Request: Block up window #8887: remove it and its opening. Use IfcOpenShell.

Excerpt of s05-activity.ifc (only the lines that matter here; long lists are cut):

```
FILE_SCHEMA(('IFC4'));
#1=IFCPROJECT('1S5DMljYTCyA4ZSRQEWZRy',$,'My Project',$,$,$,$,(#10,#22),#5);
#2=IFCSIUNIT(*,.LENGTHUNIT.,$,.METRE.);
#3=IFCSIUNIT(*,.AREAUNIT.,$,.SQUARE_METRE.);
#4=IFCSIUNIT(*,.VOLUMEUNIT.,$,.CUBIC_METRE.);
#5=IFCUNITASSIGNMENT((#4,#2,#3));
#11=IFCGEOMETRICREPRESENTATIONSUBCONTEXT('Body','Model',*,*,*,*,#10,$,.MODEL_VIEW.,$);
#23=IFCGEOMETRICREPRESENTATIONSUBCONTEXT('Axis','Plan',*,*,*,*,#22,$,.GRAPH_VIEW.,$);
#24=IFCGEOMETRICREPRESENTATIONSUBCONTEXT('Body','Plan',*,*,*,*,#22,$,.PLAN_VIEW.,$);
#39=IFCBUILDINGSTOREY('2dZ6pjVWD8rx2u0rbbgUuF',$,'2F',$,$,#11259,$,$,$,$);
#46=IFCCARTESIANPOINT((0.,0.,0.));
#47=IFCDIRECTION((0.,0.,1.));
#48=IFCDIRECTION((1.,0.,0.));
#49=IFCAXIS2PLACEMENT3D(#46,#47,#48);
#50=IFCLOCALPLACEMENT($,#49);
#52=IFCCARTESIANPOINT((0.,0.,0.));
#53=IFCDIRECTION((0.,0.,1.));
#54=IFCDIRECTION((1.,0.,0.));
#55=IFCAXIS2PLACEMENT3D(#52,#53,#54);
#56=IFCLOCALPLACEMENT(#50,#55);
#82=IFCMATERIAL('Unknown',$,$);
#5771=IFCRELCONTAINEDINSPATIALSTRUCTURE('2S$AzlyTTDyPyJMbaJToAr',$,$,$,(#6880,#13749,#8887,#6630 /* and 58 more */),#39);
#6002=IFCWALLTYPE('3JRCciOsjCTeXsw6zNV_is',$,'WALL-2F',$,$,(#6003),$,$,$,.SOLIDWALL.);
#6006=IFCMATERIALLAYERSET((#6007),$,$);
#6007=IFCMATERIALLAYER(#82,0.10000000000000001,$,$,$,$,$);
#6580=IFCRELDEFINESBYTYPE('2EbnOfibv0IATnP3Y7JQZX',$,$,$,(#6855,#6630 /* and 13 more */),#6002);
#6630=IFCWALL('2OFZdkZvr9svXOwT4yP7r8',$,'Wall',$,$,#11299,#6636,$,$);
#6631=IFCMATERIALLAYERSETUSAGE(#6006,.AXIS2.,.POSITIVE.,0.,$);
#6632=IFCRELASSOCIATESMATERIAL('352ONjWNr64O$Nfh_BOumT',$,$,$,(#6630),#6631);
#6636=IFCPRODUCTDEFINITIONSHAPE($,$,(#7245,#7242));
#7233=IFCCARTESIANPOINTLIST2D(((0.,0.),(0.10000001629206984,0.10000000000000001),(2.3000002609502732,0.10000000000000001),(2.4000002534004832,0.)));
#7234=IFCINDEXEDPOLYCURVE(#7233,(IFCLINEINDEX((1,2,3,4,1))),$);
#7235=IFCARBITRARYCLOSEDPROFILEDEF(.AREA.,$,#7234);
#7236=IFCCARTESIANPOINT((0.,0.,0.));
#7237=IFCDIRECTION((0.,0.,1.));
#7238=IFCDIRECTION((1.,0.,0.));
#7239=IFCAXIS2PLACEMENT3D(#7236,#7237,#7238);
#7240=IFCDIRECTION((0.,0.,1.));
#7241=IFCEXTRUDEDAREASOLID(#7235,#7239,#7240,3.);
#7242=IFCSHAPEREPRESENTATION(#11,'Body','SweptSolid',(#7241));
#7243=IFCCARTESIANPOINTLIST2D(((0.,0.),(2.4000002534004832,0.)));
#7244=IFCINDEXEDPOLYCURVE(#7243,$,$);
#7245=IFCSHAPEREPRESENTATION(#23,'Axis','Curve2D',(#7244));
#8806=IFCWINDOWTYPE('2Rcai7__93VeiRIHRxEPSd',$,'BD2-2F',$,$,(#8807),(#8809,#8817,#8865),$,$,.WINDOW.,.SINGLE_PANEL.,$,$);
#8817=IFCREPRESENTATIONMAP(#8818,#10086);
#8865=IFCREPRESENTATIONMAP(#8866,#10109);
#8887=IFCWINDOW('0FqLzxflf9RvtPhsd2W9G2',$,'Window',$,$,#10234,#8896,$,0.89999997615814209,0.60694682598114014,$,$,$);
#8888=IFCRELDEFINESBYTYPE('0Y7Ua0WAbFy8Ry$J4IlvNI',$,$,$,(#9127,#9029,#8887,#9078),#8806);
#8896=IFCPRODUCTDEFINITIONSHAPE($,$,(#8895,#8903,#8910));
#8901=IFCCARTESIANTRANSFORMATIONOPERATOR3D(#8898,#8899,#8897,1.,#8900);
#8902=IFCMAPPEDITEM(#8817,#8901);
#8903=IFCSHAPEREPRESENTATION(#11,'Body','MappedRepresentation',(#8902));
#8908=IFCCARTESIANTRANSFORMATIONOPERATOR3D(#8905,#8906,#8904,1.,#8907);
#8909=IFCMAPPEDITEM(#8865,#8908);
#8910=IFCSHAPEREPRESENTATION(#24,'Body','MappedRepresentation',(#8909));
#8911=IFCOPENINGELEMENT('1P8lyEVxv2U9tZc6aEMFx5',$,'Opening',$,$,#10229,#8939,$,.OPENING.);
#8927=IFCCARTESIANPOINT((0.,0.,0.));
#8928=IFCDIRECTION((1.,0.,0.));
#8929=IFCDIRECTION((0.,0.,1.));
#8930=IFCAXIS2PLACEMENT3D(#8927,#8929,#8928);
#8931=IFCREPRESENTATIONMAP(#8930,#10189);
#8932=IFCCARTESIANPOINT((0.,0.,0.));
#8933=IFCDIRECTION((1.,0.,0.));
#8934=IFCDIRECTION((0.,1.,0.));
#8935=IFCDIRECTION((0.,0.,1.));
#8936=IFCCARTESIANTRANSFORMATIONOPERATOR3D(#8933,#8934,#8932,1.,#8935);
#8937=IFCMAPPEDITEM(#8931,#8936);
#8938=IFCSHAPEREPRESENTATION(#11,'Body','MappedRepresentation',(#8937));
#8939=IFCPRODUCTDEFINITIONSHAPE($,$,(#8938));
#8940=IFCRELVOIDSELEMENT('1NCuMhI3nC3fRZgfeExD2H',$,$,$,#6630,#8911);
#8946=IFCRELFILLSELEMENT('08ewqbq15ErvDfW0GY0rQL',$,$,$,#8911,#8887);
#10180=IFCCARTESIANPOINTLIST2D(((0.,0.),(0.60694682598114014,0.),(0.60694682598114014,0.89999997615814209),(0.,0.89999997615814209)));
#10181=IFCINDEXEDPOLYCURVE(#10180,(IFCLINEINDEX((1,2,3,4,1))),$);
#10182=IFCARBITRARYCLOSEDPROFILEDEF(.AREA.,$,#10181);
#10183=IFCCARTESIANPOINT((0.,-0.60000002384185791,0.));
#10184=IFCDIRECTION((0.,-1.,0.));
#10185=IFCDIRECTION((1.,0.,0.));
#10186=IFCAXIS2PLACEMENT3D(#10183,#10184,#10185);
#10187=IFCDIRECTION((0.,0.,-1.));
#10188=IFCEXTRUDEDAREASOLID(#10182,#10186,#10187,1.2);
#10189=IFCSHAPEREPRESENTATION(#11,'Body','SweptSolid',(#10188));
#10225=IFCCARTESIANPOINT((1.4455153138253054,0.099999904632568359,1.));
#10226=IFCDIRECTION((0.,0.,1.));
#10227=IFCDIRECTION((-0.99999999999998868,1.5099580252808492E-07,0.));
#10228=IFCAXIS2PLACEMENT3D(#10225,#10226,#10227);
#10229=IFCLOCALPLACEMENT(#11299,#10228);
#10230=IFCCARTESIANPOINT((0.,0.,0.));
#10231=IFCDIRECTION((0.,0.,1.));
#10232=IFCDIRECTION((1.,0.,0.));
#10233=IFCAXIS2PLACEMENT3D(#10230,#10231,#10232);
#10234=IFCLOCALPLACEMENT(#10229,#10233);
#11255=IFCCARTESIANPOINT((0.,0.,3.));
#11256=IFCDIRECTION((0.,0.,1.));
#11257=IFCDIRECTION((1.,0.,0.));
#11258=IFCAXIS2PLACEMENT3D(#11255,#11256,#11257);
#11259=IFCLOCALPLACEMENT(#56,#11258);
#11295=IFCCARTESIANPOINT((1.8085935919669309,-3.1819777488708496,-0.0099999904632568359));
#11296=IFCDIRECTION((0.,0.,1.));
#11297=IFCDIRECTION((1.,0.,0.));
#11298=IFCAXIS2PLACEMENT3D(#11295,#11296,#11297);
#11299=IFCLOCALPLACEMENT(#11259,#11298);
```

```python
import ifcopenshell
import ifcopenshell.api.feature
import ifcopenshell.api.root
import ifcopenshell.geom
import ifcopenshell.util.shape

model = ifcopenshell.open("s05-activity.ifc")
settings = ifcopenshell.geom.settings()


def volume(element):
    """Net volume in cubic metres, openings subtracted."""
    shape = ifcopenshell.geom.create_shape(settings, element)
    return ifcopenshell.util.shape.get_volume(shape.geometry)


window = model.by_guid("0FqLzxflf9RvtPhsd2W9G2")
opening = window.FillsVoids[0].RelatingOpeningElement
wall = opening.VoidsElements[0].RelatingBuildingElement
before = volume(wall)

ifcopenshell.api.root.remove_product(model, product=window)
ifcopenshell.api.feature.remove_feature(model, feature=opening)

after = volume(wall)

print(f"wall volume {before:.3f} -> {after:.3f} m3")

model.write("s05-activity_v2.ifc")
```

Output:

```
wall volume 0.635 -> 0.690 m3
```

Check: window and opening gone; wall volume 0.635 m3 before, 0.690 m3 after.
